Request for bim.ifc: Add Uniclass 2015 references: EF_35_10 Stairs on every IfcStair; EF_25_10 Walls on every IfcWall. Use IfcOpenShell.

First a look at what the model holds.

```python
import ifcopenshell

model = ifcopenshell.open("bim.ifc")
print(model.schema)
print("classifications:", [c.Name for c in model.by_type("IfcClassification")])
for ifc_class in ("IfcDoor", "IfcRoof", "IfcStair", "IfcWall", "IfcWindow"):
    print(ifc_class, len(model.by_type(ifc_class)))
```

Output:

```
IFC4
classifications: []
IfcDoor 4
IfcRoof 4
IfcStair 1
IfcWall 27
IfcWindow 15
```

```python
import ifcopenshell
import ifcopenshell.api.classification

model = ifcopenshell.open("bim.ifc")

system = ifcopenshell.api.classification.add_classification(model, classification="Uniclass 2015")

codes = {
    "IfcStair": ("EF_35_10", "Stairs"),
    "IfcWall": ("EF_25_10", "Walls"),
}
for ifc_class, (code, name) in codes.items():
    products = model.by_type(ifc_class)
    ifcopenshell.api.classification.add_reference(
        model, products=products, classification=system, identification=code, name=name
    )
    print(code, len(products))

model.write("bim_rev.ifc")
```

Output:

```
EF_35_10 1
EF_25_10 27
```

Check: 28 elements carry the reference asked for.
